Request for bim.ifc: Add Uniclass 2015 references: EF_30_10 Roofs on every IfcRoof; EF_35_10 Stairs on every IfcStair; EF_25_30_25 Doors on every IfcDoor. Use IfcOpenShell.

First a look at what the model holds.

```python
import ifcopenshell

model = ifcopenshell.open("bim.ifc")
print(model.schema)
print("classifications:", [c.Name for c in model.by_type("IfcClassification")])
for ifc_class in ("IfcDoor", "IfcRoof", "IfcStair", "IfcWall", "IfcWindow"):
    print(ifc_class, len(model.by_type(ifc_class)))
```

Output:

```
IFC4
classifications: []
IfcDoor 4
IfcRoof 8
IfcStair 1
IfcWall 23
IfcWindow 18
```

```python
import ifcopenshell
import ifcopenshell.api.classification

model = ifcopenshell.open("bim.ifc")

system = ifcopenshell.api.classification.add_classification(model, classification="Uniclass 2015")

codes = {
    "IfcRoof": ("EF_30_10", "Roofs"),
    "IfcStair": ("EF_35_10", "Stairs"),
    "IfcDoor": ("EF_25_30_25", "Doors"),
}
for ifc_class, (code, name) in codes.items():
    products = model.by_type(ifc_class)
    ifcopenshell.api.classification.add_reference(
        model, products=products, classification=system, identification=code, name=name
    )
    print(code, len(products))

model.write("bim-out.ifc")
```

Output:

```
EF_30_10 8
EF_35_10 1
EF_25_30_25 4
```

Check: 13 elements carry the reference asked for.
